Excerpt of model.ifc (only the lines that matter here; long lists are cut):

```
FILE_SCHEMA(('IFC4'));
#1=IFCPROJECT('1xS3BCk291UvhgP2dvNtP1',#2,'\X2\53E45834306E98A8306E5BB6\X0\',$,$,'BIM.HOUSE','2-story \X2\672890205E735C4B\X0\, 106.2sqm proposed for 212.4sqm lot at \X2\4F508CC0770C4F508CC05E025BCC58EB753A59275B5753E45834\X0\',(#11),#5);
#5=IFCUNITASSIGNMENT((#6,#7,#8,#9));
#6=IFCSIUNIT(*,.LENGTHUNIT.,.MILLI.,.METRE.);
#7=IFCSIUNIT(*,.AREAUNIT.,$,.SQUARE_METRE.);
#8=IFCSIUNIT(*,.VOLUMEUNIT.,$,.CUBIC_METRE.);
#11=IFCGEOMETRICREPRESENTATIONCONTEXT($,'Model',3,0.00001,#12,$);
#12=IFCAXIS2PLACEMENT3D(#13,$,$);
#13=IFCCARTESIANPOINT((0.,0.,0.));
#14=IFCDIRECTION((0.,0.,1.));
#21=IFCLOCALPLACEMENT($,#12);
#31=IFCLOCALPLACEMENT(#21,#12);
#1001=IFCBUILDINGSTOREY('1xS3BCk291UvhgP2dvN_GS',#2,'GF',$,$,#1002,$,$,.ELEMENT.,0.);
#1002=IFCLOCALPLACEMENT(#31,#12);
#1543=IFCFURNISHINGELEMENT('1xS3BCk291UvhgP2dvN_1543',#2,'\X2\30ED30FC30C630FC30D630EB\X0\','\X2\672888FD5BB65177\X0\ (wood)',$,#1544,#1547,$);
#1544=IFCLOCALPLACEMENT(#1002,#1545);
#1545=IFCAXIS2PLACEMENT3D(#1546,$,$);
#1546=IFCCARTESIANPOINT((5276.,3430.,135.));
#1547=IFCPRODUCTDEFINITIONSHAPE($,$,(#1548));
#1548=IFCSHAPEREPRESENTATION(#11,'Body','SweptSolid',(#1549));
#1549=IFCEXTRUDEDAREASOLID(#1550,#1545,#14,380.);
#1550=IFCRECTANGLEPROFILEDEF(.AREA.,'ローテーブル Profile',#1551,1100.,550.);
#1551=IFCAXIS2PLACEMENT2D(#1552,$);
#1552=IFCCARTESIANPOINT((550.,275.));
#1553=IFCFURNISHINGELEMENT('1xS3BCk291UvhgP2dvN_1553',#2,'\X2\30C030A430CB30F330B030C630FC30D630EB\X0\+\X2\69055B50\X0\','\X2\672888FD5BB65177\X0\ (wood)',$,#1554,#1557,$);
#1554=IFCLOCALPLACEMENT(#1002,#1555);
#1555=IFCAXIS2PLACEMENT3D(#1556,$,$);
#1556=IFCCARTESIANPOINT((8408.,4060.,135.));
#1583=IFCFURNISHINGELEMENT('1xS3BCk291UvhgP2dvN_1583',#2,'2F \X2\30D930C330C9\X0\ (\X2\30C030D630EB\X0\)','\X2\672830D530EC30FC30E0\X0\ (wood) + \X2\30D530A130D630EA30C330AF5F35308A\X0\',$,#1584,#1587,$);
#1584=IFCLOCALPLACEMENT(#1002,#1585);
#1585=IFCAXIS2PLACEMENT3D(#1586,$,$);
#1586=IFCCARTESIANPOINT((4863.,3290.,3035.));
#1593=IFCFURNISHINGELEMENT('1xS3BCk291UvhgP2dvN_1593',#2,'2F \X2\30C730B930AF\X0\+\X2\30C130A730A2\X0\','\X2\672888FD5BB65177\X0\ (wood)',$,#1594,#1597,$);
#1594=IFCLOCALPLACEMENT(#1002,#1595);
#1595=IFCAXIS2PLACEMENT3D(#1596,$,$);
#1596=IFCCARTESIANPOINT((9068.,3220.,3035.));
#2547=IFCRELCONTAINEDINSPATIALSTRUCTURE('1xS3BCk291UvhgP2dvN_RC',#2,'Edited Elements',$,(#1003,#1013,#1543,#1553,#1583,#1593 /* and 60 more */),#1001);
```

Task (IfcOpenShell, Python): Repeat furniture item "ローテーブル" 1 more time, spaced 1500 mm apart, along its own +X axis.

```python
import ifcopenshell
import ifcopenshell.api.geometry
import ifcopenshell.api.root
import ifcopenshell.util.element
import ifcopenshell.util.placement
import ifcopenshell.util.unit

model = ifcopenshell.open("model.ifc")
unit_scale = ifcopenshell.util.unit.calculate_unit_scale(model)


def reuse_history(source, copy):
    """copy_class also copies each property set's owner history, people and application; keep the originals."""
    for rel in copy.IsDefinedBy:
        if rel.is_a("IfcRelDefinesByProperties") and (history := rel.RelatingPropertyDefinition.OwnerHistory):
            rel.RelatingPropertyDefinition.OwnerHistory = source.OwnerHistory
            ifcopenshell.util.element.remove_deep2(model, history)


source = model.by_guid("1xS3BCk291UvhgP2dvN_1543")
base = ifcopenshell.util.placement.get_local_placement(source.ObjectPlacement)
step = base[:3, 0] * 1.5 / unit_scale

for i in range(1, 2):
    copy = ifcopenshell.api.root.copy_class(model, product=source)
    copy.Representation = ifcopenshell.util.element.copy_deep(
        model, source.Representation, exclude=["IfcGeometricRepresentationContext", "IfcRepresentationMap"]
    )
    reuse_history(source, copy)
    matrix = base.copy()
    matrix[:3, 3] += i * step
    print("added at", matrix[:3, 3].round(3) + 0.0)
    ifcopenshell.api.geometry.edit_object_placement(model, product=copy, matrix=matrix, is_si=False)

model.write("model_v2.ifc")
```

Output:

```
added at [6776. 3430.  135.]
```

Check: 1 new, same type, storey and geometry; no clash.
